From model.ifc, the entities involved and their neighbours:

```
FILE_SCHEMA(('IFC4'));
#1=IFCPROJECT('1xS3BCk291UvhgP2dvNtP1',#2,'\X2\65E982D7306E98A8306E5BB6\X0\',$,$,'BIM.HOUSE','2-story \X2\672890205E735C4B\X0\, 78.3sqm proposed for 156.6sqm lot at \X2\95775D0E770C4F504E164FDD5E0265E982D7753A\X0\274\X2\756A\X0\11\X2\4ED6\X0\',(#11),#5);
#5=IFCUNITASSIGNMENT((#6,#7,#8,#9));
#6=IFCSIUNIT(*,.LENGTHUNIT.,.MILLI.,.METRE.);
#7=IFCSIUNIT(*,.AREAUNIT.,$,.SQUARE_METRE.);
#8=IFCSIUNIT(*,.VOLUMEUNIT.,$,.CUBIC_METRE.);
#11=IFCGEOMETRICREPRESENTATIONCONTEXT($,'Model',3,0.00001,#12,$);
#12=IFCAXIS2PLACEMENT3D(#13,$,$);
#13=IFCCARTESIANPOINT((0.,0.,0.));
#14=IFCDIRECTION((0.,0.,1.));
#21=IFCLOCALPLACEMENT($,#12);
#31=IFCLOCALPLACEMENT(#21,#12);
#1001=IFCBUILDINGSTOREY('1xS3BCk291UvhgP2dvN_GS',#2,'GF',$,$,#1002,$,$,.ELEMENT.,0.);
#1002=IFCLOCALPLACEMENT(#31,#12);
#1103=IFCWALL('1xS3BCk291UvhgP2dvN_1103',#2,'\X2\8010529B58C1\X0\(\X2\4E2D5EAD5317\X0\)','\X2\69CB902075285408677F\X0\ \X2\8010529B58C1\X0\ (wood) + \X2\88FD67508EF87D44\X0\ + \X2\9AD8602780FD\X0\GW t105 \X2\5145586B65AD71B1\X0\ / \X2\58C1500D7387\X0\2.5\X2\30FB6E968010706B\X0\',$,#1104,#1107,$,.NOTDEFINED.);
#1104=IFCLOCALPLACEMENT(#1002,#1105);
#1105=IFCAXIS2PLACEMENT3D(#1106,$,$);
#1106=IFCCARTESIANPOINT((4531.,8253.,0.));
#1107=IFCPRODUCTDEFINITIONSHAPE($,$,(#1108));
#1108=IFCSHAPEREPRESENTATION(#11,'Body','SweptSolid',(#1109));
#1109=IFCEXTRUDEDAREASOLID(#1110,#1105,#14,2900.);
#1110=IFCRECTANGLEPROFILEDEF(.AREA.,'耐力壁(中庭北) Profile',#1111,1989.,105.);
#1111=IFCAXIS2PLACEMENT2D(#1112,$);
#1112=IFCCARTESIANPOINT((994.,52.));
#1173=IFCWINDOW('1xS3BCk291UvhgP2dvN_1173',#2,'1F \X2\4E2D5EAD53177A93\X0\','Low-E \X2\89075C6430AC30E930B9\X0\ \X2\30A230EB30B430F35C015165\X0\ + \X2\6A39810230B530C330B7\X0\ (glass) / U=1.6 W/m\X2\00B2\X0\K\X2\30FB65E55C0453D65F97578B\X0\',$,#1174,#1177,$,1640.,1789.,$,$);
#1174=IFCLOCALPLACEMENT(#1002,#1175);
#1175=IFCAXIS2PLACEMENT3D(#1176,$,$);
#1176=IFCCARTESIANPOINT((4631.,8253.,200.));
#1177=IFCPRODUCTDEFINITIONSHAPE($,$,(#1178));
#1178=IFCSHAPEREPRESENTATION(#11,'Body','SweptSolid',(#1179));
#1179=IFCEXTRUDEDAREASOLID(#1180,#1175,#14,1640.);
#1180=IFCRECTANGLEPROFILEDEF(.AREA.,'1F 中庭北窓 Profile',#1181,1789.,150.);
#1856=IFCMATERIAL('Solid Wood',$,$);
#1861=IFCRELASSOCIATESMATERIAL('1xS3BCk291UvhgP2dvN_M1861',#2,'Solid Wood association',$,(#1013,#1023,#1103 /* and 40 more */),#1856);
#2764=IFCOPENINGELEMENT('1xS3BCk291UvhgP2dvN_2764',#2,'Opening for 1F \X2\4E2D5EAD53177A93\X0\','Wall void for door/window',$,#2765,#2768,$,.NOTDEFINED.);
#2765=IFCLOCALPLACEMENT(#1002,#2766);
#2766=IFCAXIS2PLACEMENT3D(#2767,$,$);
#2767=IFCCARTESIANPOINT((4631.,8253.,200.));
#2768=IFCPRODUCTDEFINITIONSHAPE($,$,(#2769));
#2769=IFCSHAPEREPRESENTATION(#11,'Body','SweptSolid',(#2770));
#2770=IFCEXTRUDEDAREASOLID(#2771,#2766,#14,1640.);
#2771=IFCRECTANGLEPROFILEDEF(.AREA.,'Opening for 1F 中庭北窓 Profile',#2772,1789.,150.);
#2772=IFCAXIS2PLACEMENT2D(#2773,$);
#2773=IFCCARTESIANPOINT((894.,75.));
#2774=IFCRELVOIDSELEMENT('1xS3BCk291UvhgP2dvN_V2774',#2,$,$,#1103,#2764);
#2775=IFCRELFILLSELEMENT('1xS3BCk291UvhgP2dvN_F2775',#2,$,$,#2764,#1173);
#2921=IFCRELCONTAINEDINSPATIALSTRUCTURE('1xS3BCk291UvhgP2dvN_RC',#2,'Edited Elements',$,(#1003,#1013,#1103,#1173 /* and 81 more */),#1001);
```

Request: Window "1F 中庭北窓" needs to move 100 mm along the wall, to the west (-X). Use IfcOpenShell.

```python
import ifcopenshell
import ifcopenshell.api.geometry
import ifcopenshell.util.placement
import ifcopenshell.util.unit

model = ifcopenshell.open("model.ifc")
unit_scale = ifcopenshell.util.unit.calculate_unit_scale(model)

window = model.by_guid("1xS3BCk291UvhgP2dvN_1173")
opening = window.FillsVoids[0].RelatingOpeningElement
wall = opening.VoidsElements[0].RelatingBuildingElement

wall_matrix = ifcopenshell.util.placement.get_local_placement(wall.ObjectPlacement)
shift = wall_matrix[:3, 0] * -0.1 / unit_scale
before = ifcopenshell.util.placement.get_local_placement(window.ObjectPlacement)[:3, 3].copy()

# The window is not placed relative to its opening, so move both.
for product in (opening, window):
    matrix = ifcopenshell.util.placement.get_local_placement(product.ObjectPlacement)
    matrix[:3, 3] += shift
    ifcopenshell.api.geometry.edit_object_placement(model, product=product, matrix=matrix, is_si=False)

after = ifcopenshell.util.placement.get_local_placement(window.ObjectPlacement)[:3, 3]
print("window moved by", (after - before).round(3) + 0.0)

model.write("model_edited.ifc")
```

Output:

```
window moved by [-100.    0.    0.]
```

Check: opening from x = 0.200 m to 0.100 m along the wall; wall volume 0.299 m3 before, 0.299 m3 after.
